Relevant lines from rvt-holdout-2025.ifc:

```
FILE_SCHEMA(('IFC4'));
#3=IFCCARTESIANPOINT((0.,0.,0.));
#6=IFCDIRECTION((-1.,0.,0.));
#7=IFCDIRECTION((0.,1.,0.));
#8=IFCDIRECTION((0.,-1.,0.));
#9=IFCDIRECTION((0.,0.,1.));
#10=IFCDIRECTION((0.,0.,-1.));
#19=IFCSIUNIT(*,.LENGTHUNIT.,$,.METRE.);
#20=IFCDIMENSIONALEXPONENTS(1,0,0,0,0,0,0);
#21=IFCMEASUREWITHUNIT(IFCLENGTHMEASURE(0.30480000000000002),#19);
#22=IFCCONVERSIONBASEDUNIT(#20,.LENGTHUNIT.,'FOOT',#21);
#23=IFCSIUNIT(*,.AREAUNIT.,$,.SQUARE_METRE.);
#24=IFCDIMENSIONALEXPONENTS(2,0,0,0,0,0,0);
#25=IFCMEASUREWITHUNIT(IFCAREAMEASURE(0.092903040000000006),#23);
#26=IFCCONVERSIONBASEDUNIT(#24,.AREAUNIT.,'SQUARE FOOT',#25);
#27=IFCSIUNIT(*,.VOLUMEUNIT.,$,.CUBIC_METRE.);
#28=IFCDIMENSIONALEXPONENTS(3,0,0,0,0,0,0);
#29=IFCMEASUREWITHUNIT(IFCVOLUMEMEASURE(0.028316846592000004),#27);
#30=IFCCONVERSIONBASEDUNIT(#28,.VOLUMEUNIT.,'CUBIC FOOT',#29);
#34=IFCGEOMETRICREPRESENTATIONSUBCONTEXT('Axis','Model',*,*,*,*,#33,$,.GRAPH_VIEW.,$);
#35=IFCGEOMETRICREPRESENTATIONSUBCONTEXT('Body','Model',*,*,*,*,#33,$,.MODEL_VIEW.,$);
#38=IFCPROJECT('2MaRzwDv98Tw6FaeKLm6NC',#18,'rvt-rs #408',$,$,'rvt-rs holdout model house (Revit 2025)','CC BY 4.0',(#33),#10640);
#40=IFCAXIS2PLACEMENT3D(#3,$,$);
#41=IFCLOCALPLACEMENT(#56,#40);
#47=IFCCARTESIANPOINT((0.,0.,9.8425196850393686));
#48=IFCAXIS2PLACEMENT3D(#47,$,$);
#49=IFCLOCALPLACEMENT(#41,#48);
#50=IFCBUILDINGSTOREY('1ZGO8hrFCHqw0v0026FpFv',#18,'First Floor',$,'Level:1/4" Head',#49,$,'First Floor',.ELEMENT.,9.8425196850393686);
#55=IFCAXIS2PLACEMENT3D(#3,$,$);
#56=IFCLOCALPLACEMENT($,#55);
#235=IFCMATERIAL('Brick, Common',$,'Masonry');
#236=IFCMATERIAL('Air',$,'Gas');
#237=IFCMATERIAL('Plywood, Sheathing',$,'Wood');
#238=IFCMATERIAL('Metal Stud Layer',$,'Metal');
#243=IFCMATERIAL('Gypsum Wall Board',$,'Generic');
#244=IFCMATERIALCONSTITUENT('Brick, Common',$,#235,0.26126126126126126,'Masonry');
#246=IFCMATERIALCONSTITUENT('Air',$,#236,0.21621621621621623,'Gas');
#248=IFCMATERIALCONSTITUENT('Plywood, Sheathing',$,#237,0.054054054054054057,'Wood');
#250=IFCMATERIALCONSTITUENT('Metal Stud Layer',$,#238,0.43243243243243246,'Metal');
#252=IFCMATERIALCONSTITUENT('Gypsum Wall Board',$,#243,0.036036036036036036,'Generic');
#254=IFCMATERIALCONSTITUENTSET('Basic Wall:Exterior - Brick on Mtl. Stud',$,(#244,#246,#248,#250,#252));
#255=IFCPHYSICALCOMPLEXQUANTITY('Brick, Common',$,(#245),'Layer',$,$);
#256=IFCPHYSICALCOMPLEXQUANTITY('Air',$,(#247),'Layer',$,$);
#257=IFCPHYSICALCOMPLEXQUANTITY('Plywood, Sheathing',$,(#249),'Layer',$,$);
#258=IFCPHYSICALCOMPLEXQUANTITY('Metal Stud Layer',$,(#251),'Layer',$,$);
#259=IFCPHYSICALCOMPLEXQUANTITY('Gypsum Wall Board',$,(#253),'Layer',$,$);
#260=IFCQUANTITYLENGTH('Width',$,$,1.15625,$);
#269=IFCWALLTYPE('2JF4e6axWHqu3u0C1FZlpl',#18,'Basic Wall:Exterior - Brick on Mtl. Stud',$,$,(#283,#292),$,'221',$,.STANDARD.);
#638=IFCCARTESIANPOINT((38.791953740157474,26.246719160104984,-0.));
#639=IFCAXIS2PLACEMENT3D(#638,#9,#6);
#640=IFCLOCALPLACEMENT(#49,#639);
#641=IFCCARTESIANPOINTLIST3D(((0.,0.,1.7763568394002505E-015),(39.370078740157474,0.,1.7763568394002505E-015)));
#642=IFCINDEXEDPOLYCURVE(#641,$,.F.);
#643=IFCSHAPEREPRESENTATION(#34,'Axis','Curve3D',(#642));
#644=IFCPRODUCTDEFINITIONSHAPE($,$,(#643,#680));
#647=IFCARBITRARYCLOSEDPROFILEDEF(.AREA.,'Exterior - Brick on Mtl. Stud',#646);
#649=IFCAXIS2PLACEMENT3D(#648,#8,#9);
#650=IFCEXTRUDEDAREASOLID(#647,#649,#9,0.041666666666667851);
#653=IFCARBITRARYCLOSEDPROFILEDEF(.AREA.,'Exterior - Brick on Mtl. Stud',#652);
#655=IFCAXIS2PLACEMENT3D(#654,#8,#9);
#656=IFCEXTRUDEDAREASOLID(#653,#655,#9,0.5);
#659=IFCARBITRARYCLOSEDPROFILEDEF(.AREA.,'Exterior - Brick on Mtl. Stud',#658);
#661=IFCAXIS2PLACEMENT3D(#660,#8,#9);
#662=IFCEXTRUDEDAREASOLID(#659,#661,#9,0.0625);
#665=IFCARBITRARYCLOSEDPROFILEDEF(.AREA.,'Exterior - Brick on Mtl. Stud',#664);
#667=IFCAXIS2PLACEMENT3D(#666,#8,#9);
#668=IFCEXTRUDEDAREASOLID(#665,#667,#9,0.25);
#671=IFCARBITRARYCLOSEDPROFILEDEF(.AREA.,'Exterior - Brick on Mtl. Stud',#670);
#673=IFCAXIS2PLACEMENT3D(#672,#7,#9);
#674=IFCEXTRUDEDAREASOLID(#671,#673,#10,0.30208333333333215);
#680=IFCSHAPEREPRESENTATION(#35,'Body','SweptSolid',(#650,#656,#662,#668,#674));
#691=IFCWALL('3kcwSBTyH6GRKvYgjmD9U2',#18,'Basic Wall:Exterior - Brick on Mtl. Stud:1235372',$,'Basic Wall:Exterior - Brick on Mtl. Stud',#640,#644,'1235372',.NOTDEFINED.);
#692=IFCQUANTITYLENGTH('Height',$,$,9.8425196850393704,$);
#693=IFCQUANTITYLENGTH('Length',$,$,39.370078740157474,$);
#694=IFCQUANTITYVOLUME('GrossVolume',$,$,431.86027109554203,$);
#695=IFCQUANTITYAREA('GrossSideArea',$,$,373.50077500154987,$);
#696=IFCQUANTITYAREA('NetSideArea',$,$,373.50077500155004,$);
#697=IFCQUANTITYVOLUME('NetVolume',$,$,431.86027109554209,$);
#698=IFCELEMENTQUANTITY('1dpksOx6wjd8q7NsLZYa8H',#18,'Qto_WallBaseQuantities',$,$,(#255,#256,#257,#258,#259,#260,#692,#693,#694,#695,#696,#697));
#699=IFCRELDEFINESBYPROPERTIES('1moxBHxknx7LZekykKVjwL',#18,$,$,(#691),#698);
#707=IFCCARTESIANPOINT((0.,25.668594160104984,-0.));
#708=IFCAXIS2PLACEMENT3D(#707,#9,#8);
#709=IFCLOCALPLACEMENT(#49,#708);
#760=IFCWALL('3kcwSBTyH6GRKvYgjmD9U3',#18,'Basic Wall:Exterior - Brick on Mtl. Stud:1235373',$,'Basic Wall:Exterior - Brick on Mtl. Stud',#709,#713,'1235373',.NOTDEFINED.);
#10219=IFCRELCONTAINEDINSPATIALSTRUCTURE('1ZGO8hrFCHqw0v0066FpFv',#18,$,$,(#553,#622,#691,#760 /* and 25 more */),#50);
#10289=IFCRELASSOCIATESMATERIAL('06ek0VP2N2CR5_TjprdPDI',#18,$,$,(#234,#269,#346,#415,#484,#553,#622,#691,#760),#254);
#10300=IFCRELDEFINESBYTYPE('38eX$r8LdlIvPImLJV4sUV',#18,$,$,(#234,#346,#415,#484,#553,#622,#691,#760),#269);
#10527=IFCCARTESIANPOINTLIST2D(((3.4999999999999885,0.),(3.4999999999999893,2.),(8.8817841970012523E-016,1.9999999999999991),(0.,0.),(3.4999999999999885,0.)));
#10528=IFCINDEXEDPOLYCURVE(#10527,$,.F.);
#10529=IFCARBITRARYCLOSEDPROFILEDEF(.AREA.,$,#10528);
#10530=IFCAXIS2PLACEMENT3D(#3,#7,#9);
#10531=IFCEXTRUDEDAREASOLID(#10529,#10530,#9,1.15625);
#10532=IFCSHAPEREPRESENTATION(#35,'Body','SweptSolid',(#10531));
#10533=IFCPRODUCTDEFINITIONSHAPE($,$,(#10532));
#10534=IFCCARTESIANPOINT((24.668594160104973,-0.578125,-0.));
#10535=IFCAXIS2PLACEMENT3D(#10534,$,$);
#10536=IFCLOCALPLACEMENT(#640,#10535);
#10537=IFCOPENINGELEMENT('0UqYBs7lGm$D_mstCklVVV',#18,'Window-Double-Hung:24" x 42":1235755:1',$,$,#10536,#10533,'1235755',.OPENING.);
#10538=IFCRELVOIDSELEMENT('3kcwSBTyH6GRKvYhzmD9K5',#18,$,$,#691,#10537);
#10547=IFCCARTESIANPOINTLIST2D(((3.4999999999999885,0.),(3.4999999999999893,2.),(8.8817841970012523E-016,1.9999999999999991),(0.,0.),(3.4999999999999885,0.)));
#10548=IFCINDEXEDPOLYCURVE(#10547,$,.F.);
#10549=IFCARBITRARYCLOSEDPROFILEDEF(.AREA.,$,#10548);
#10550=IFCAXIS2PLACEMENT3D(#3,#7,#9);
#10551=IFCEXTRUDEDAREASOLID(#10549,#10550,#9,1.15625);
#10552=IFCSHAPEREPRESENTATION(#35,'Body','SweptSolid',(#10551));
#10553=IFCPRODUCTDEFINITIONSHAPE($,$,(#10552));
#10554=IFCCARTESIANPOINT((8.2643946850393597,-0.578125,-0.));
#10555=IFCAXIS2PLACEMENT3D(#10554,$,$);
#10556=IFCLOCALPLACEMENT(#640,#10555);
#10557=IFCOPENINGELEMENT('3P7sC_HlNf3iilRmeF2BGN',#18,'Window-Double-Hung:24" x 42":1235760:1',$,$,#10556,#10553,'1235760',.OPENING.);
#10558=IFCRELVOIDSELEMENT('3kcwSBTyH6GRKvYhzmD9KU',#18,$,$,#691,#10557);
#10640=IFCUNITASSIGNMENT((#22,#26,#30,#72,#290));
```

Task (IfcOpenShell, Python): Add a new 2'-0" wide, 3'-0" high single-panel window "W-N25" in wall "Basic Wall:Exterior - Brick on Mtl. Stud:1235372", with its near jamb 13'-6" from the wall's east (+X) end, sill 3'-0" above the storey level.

```python
import numpy as np
import ifcopenshell
import ifcopenshell.api.feature
import ifcopenshell.api.geometry
import ifcopenshell.api.pset
import ifcopenshell.api.root
import ifcopenshell.api.spatial
import ifcopenshell.geom
import ifcopenshell.util.element
import ifcopenshell.util.placement
import ifcopenshell.util.representation
import ifcopenshell.util.shape
import ifcopenshell.util.unit

model = ifcopenshell.open("rvt-holdout-2025.ifc")
unit_scale = ifcopenshell.util.unit.calculate_unit_scale(model)
area_scale = ifcopenshell.util.unit.calculate_unit_scale(model, "AREAUNIT")
volume_scale = ifcopenshell.util.unit.calculate_unit_scale(model, "VOLUMEUNIT")
settings = ifcopenshell.geom.settings()


def volume(element):
    """Net volume in cubic metres, openings subtracted."""
    shape = ifcopenshell.geom.create_shape(settings, element)
    return ifcopenshell.util.shape.get_volume(shape.geometry)


wall = model.by_guid("3kcwSBTyH6GRKvYgjmD9U2")
storey = ifcopenshell.util.element.get_container(wall, ifc_class="IfcBuildingStorey")
context = ifcopenshell.util.representation.get_context(model, "Model", "Body", "MODEL_VIEW")
before = volume(wall)

width, height, from_end, sill = 0.6096, 0.9144, 4.1148, 0.9144  # metres

# The wall runs along its own X axis, and the end named is its -X end.
wall_shape = ifcopenshell.geom.create_shape(settings, wall)
x, y, z = ifcopenshell.util.shape.get_vertices(wall_shape.geometry).T
start = x.min() + from_end
face, thickness = float(y.min()), float(y.max() - y.min())
wall_matrix = ifcopenshell.util.placement.get_local_placement(wall.ObjectPlacement)
level = ifcopenshell.util.placement.get_local_placement(storey.ObjectPlacement)[2, 3]


def in_wall(x, y):
    """Placement at x, y metres in the wall's axes, at sill height."""
    matrix = wall_matrix.copy()
    matrix[:, 3] = wall_matrix @ np.array([x / unit_scale, y / unit_scale, 0.0, 1.0])
    matrix[2, 3] = level + sill / unit_scale
    return matrix


# Opening: a box that overshoots both wall faces by 50 mm.
opening = ifcopenshell.api.root.create_entity(model, ifc_class="IfcOpeningElement", predefined_type="OPENING")
box = ifcopenshell.api.geometry.add_wall_representation(
    model, context=context, length=width, height=height, thickness=thickness + 0.1
)
ifcopenshell.api.geometry.assign_representation(model, product=opening, representation=box)
ifcopenshell.api.geometry.edit_object_placement(model, product=opening, matrix=in_wall(start, face - 0.05), is_si=False)
ifcopenshell.api.feature.add_feature(model, feature=opening, element=wall)

window = ifcopenshell.api.root.create_entity(model, ifc_class="IfcWindow", name="W-N25", predefined_type="WINDOW")
window.OverallWidth, window.OverallHeight = width / unit_scale, height / unit_scale
window.PartitioningType = "SINGLE_PANEL"
body = ifcopenshell.api.geometry.add_window_representation(
    model,
    context=context,
    overall_width=window.OverallWidth,
    overall_height=window.OverallHeight,
    partition_type="SINGLE_PANEL",
)
ifcopenshell.api.geometry.assign_representation(model, product=window, representation=body)
ifcopenshell.api.spatial.assign_container(model, products=[window], relating_structure=storey)
ifcopenshell.api.feature.add_filling(model, opening=opening, element=window)

# Centre the window in the wall's thickness.
ifcopenshell.api.geometry.edit_object_placement(model, product=window, matrix=in_wall(start, face), is_si=False)
window_shape = ifcopenshell.geom.create_shape(settings, window)
depth = ifcopenshell.util.shape.get_vertices(window_shape.geometry)[:, 1]
offset = face + thickness / 2 - (depth.min() + depth.max()) / 2
ifcopenshell.api.geometry.edit_object_placement(model, product=window, matrix=in_wall(start, offset), is_si=False)

after = volume(wall)

# Update the wall's stored quantities.
qto = model.by_id(ifcopenshell.util.element.get_pset(wall, "Qto_WallBaseQuantities", should_inherit=False)["id"])
ifcopenshell.api.pset.edit_qto(model, qto=qto, properties={
    "NetSideArea": after / thickness / area_scale,
    "NetVolume": after / volume_scale,
})

print(f"wall volume {before:.3f} -> {after:.3f} m3")

model.write("rvt-holdout-2025_updated.ifc")
```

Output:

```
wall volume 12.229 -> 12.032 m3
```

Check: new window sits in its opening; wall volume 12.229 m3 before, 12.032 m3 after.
